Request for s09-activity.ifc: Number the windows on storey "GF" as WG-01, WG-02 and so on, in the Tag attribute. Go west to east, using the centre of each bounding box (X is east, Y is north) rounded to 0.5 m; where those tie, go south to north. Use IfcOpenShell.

First a look at what the model holds.

```python
import ifcopenshell
import ifcopenshell.util.element
import ifcopenshell.util.placement

model = ifcopenshell.open("s09-activity.ifc")
print(model.schema)
storey = next(s for s in model.by_type("IfcBuildingStorey") if s.Name == "GF")
windows = [e for e in ifcopenshell.util.element.get_decomposition(storey) if e.is_a("IfcWindow")]
for e in sorted(windows, key=lambda e: e.id()):
    origin = ifcopenshell.util.placement.get_local_placement(e.ObjectPlacement)[:3, 3]
    print(e.id(), e.Tag, e.Name, origin.round(2) + 0.0, sep=" | ")
```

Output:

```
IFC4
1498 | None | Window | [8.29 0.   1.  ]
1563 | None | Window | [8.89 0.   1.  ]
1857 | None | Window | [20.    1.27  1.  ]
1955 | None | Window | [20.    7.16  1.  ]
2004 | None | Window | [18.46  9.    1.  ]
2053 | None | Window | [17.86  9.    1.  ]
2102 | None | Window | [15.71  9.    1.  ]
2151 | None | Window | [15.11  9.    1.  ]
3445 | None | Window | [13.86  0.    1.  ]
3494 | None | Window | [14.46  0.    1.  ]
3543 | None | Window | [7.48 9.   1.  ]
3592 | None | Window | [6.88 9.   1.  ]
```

```python
import ifcopenshell
import ifcopenshell.geom
import ifcopenshell.util.element
import ifcopenshell.util.shape

model = ifcopenshell.open("s09-activity.ifc")
settings = ifcopenshell.geom.settings()
settings.set("use-world-coords", True)


def centre(element):
    shape = ifcopenshell.geom.create_shape(settings, element)
    return ifcopenshell.util.shape.get_bbox_centroid(shape.geometry)


storey = next(s for s in model.by_type("IfcBuildingStorey") if s.Name == "GF")
windows = [e for e in ifcopenshell.util.element.get_decomposition(storey) if e.is_a("IfcWindow")]

# Insertion points can sit at a corner or the storey origin, so sort by the geometry (in metres).
centres = {e: centre(e) for e in windows}
windows.sort(key=lambda e: (round(centres[e][0] / 0.5), centres[e][1]))

for i, e in enumerate(windows, start=1):
    number = f"WG-{i:02d}"
    e.Tag = number
    print(e.id(), number)

model.write("s09-activity-out.ifc")
```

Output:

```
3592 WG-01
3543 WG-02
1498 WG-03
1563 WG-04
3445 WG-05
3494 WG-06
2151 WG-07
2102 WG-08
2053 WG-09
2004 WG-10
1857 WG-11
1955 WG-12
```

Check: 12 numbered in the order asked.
